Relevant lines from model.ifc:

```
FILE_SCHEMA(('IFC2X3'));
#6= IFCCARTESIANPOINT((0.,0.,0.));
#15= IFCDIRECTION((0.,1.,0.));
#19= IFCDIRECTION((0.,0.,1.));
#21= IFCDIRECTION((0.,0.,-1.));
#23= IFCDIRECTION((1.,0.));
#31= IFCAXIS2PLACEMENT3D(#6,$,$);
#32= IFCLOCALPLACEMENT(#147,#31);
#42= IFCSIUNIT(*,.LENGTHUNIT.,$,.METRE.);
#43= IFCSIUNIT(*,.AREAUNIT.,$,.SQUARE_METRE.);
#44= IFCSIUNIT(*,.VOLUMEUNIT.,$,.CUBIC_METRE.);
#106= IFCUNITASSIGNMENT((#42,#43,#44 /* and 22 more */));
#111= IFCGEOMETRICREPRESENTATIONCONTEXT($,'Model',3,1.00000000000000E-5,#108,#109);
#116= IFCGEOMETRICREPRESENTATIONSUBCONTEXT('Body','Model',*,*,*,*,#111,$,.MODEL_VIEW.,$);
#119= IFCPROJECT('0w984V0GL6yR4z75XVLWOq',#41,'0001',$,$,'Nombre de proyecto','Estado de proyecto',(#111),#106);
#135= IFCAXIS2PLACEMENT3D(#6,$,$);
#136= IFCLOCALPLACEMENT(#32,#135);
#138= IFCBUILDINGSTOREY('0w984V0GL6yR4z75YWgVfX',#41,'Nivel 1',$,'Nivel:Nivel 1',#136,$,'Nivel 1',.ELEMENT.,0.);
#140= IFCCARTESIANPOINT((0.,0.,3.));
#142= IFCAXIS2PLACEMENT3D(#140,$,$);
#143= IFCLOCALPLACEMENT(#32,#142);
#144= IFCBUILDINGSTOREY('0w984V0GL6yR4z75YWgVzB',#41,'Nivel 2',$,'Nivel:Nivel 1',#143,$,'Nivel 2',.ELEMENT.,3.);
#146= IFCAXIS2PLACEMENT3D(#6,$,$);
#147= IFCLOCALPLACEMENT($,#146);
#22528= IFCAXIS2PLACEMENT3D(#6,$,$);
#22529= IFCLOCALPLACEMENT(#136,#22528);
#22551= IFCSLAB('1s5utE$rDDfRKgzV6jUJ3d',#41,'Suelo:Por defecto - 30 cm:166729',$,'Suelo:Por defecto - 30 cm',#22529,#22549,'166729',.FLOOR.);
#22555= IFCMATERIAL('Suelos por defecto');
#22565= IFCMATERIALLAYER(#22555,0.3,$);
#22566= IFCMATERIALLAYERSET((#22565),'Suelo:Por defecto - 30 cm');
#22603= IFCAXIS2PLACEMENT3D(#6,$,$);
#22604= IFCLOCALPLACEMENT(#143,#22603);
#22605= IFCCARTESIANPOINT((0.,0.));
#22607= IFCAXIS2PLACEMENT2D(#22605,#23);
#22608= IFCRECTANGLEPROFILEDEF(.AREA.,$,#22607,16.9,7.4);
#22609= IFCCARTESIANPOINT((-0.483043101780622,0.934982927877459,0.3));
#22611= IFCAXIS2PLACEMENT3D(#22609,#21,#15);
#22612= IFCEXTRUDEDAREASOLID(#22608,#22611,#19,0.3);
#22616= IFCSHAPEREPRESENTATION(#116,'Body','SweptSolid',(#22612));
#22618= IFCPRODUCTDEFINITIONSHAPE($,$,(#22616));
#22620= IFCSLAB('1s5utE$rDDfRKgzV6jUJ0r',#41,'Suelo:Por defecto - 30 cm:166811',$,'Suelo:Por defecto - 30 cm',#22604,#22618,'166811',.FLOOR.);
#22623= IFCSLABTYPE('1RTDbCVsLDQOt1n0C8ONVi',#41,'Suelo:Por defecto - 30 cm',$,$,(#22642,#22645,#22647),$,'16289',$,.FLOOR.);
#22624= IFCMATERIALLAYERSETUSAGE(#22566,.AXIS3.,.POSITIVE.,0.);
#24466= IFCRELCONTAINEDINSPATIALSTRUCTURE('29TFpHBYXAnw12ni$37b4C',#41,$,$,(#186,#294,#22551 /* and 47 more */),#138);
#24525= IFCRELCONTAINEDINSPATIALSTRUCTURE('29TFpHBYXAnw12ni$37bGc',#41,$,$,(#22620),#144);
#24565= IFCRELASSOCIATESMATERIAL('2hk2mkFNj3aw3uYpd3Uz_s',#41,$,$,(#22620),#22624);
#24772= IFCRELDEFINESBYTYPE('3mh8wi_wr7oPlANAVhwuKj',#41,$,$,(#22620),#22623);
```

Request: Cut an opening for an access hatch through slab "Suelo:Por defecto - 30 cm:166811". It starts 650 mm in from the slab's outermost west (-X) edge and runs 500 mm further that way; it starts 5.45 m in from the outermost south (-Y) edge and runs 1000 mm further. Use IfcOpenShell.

```python
import numpy as np
import ifcopenshell
import ifcopenshell.api.feature
import ifcopenshell.api.geometry
import ifcopenshell.api.root
import ifcopenshell.geom
import ifcopenshell.util.placement
import ifcopenshell.util.representation
import ifcopenshell.util.shape
import ifcopenshell.util.unit

model = ifcopenshell.open("model.ifc")
unit_scale = ifcopenshell.util.unit.calculate_unit_scale(model)
settings = ifcopenshell.geom.settings()


def volume(element):
    """Net volume in cubic metres, openings subtracted."""
    shape = ifcopenshell.geom.create_shape(settings, element)
    return ifcopenshell.util.shape.get_volume(shape.geometry)


slab = model.by_id(22620)
before = volume(slab)

# Extent in the slab's own axes, in metres. The edges named are its -X and -Y sides.
slab_shape = ifcopenshell.geom.create_shape(settings, slab)
vertices = ifcopenshell.util.shape.get_vertices(slab_shape.geometry)
x_min, y_min, bottom = vertices.min(axis=0)
top = vertices[:, 2].max()

opening = ifcopenshell.api.root.create_entity(model, ifc_class="IfcOpeningElement", name="Access hatch opening")
context = ifcopenshell.util.representation.get_context(model, "Model", "Body", "MODEL_VIEW")
width, depth = 0.5, 1
outline = [(0.0, 0.0), (width, 0.0), (width, depth), (0.0, depth), (0.0, 0.0)]
# Overshoot both faces by 50 mm so the cut is clean.
shape = ifcopenshell.api.geometry.add_slab_representation(
    model, context=context, depth=top - bottom + 0.1, polyline=outline
)
ifcopenshell.api.geometry.assign_representation(model, product=opening, representation=shape)

matrix = ifcopenshell.util.placement.get_local_placement(slab.ObjectPlacement)
matrix[:, 3] = matrix @ np.append(np.array([x_min + 0.65, y_min + 5.45, bottom - 0.05]) / unit_scale, 1.0)
ifcopenshell.api.geometry.edit_object_placement(model, product=opening, matrix=matrix, is_si=False)
ifcopenshell.api.feature.add_feature(model, feature=opening, element=slab)

after = volume(slab)

print(f"slab volume {before:.3f} -> {after:.3f} m3")

model.write("model_updated.ifc")
```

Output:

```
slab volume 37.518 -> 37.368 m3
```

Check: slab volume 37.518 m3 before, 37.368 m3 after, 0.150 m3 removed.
